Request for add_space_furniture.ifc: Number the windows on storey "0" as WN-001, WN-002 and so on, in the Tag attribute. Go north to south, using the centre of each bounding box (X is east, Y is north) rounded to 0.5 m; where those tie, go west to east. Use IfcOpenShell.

First a look at what the model holds.

```python
import ifcopenshell
import ifcopenshell.util.element
import ifcopenshell.util.placement

model = ifcopenshell.open("add_space_furniture.ifc")
print(model.schema)
storey = next(s for s in model.by_type("IfcBuildingStorey") if s.Name == "0")
windows = [e for e in ifcopenshell.util.element.get_decomposition(storey) if e.is_a("IfcWindow")]
for e in sorted(windows, key=lambda e: e.id()):
    origin = ifcopenshell.util.placement.get_local_placement(e.ObjectPlacement)[:3, 3]
    print(e.id(), e.Tag, e.Name, origin.round(2) + 0.0, sep=" | ")
```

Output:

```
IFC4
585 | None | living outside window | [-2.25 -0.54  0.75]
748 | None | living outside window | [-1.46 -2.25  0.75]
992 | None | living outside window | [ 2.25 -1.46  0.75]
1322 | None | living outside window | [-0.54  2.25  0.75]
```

```python
import ifcopenshell
import ifcopenshell.geom
import ifcopenshell.util.element
import ifcopenshell.util.shape

model = ifcopenshell.open("add_space_furniture.ifc")
settings = ifcopenshell.geom.settings()
settings.set("use-world-coords", True)


def centre(element):
    shape = ifcopenshell.geom.create_shape(settings, element)
    return ifcopenshell.util.shape.get_bbox_centroid(shape.geometry)


storey = next(s for s in model.by_type("IfcBuildingStorey") if s.Name == "0")
windows = [e for e in ifcopenshell.util.element.get_decomposition(storey) if e.is_a("IfcWindow")]

# Insertion points can sit at a corner or the storey origin, so sort by the geometry (in metres).
centres = {e: centre(e) for e in windows}
windows.sort(key=lambda e: (-round(centres[e][1] / 0.5), centres[e][0]))

for i, e in enumerate(windows, start=1):
    number = f"WN-0{i:02d}"
    e.Tag = number
    print(e.id(), number)

model.write("add_space_furniture_rev.ifc")
```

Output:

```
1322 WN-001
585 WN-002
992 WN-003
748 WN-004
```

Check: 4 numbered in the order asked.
